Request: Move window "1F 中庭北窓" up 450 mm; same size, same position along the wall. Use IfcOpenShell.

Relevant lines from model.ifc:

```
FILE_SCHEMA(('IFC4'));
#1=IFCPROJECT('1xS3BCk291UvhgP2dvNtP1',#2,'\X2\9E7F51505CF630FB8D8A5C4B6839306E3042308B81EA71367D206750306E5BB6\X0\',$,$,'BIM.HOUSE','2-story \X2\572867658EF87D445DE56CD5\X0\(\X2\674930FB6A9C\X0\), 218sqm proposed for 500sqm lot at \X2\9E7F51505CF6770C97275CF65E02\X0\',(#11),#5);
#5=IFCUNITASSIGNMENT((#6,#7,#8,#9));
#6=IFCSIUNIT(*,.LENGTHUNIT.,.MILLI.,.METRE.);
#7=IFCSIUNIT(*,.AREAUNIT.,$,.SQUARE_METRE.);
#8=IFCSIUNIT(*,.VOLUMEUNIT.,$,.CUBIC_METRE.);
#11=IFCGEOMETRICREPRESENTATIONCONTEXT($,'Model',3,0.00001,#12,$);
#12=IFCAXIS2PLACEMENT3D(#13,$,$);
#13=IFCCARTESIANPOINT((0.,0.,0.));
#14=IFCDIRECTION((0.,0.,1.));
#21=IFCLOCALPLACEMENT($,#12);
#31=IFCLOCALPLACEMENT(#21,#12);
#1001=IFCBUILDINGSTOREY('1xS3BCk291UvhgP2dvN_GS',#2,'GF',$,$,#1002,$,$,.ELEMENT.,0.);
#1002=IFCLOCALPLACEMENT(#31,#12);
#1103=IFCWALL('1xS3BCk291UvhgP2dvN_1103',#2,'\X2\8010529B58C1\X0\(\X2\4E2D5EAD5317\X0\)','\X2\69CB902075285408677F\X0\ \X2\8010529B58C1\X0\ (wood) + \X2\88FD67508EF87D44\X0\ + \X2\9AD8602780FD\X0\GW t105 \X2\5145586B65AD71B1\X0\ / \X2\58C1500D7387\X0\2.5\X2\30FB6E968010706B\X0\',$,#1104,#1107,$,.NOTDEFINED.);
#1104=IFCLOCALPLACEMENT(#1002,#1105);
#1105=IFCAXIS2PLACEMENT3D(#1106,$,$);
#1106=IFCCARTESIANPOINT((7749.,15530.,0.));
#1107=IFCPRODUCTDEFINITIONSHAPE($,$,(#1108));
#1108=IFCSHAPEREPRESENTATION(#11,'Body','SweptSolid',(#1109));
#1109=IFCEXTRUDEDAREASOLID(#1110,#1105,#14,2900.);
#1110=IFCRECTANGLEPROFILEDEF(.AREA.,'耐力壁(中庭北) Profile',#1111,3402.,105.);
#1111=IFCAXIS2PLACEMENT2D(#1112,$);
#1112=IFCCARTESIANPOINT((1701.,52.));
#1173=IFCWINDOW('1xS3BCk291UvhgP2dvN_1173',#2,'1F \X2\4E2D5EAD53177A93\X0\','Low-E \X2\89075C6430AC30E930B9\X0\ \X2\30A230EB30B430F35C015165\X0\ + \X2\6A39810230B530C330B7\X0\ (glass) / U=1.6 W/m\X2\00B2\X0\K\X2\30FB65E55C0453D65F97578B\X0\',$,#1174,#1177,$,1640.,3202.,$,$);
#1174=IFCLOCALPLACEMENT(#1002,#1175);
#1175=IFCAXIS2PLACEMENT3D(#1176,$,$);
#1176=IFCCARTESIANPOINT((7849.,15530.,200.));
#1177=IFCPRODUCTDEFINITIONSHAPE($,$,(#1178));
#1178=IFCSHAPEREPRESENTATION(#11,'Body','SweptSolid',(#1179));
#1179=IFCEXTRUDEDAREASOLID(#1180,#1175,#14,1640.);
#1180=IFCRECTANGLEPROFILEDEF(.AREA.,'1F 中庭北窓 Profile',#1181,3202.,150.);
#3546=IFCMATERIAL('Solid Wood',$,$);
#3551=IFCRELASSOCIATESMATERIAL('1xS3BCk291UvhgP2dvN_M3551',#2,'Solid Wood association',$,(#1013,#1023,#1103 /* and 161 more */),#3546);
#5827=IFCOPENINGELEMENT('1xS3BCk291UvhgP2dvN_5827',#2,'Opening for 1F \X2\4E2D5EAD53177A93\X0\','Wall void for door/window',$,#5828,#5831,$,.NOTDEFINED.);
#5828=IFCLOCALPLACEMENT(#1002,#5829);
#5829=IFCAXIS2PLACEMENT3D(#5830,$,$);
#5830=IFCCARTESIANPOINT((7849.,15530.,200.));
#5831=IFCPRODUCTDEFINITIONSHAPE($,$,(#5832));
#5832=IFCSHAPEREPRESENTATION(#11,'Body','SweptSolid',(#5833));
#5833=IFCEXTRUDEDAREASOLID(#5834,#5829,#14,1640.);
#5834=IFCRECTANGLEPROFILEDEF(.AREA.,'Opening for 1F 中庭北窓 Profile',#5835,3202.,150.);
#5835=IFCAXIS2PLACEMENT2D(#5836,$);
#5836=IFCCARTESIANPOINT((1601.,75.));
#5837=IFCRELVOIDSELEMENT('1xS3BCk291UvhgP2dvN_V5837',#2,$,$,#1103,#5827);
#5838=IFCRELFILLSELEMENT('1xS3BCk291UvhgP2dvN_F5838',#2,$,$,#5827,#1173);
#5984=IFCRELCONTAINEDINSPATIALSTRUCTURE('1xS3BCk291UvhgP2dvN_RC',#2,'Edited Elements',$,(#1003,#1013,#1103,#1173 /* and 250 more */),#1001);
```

```python
import numpy as np
import ifcopenshell
import ifcopenshell.api.geometry
import ifcopenshell.util.placement
import ifcopenshell.util.unit

model = ifcopenshell.open("model.ifc")
unit_scale = ifcopenshell.util.unit.calculate_unit_scale(model)

window = model.by_guid("1xS3BCk291UvhgP2dvN_1173")
opening = window.FillsVoids[0].RelatingOpeningElement
dz = 0.45 / unit_scale

shift = np.array([0.0, 0.0, dz])
# The window is not placed relative to its opening, so move both.
for product in (opening, window):
    matrix = ifcopenshell.util.placement.get_local_placement(product.ObjectPlacement)
    matrix[:3, 3] += shift
    ifcopenshell.api.geometry.edit_object_placement(model, product=product, matrix=matrix, is_si=False)

print(f"moved by {dz * unit_scale:+.3f} m")

model.write("model_edited.ifc")
```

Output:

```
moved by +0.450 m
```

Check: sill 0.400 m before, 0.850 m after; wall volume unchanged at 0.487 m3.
